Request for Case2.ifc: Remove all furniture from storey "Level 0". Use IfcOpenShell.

First a look at what the model holds.

```python
import ifcopenshell
import ifcopenshell.util.element

model = ifcopenshell.open("Case2.ifc")
print(model.schema)
storey = next(s for s in model.by_type("IfcBuildingStorey") if s.Name == "Level 0")
furniture = [e for e in ifcopenshell.util.element.get_decomposition(storey) if e.is_a("IfcFurnishingElement")]
seen = {}
for e in furniture:
    element_type = ifcopenshell.util.element.get_type(e)
    name = element_type.Name if element_type not in (None, e) else None
    seen[name] = seen.get(name, 0) + 1
for name, count in sorted(seen.items(), key=str):
    print(count, "x", name)
```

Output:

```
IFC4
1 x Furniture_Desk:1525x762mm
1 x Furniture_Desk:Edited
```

```python
import ifcopenshell
import ifcopenshell.api.root
import ifcopenshell.util.element

model = ifcopenshell.open("Case2.ifc")

storey = next(s for s in model.by_type("IfcBuildingStorey") if s.Name == "Level 0")
furniture = [e for e in ifcopenshell.util.element.get_decomposition(storey) if e.is_a("IfcFurnishingElement")]

for e in furniture:
    ifcopenshell.api.root.remove_product(model, product=e)
print(len(furniture), "removed")

model.write("Case2-out.ifc")
```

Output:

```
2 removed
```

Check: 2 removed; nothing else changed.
